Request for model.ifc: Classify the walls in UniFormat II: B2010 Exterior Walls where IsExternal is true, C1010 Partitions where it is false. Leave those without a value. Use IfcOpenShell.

First a look at what the model holds.

```python
import ifcopenshell
import ifcopenshell.util.element

model = ifcopenshell.open("model.ifc")
print(model.schema)
print("classifications:", [c.Name for c in model.by_type("IfcClassification")])
values = [ifcopenshell.util.element.get_pset(e, "Pset_WallCommon", "IsExternal") for e in model.by_type("IfcWall")]
for value in (True, False, None):
    print("IsExternal", value, values.count(value))
```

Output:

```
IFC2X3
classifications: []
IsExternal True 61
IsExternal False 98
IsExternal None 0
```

```python
import ifcopenshell
import ifcopenshell.api.classification
import ifcopenshell.util.element

model = ifcopenshell.open("model.ifc")

# IFC2X3 requires Source and Edition and has no link from the project to the system.
system = model.create_entity("IfcClassification", Source="ASTM", Edition="E1557", Name="UniFormat II")

walls = model.by_type("IfcWall")
external = {e: ifcopenshell.util.element.get_pset(e, "Pset_WallCommon", "IsExternal") for e in walls}
for flag, code, name in ((True, "B2010", "Exterior Walls"), (False, "C1010", "Partitions")):
    products = [e for e in walls if external[e] is flag]
    ifcopenshell.api.classification.add_reference(
        model, products=products, classification=system, identification=code, name=name
    )
    print(code, len(products))

model.write("model_v2.ifc")
```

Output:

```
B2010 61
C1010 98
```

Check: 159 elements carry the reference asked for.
